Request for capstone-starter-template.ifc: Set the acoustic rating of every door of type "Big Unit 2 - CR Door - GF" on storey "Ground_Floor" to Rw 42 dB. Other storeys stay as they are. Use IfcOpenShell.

First a look at what the model holds.

```python
import ifcopenshell
import ifcopenshell.util.element

model = ifcopenshell.open("capstone-starter-template.ifc")
print(model.schema)
storey = next(s for s in model.by_type("IfcBuildingStorey") if s.Name == "Ground_Floor")
doors = [e for e in ifcopenshell.util.element.get_decomposition(storey) if e.is_a("IfcDoor")]
seen = {}
for e in doors:
    element_type = ifcopenshell.util.element.get_type(e)
    key = (element_type.Name if element_type != e and element_type else None, ifcopenshell.util.element.get_pset(e, "Pset_DoorCommon", "AcousticRating"))
    seen[key] = seen.get(key, 0) + 1
for (name, value), count in sorted(seen.items(), key=str):
    print(count, "x", name, "|", value)
```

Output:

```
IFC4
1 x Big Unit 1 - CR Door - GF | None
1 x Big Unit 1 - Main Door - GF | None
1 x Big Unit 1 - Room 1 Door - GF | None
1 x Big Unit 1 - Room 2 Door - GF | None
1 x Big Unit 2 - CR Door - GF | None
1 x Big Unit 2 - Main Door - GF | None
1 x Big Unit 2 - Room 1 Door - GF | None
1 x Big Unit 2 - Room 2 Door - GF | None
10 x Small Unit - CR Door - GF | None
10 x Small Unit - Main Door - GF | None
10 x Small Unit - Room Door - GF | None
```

```python
import ifcopenshell
import ifcopenshell.api.pset
import ifcopenshell.util.element

model = ifcopenshell.open("capstone-starter-template.ifc")

storey = next(s for s in model.by_type("IfcBuildingStorey") if s.Name == "Ground_Floor")
doors = [e for e in ifcopenshell.util.element.get_decomposition(storey) if e.is_a("IfcDoor")]

count = 0
for e in doors:
    element_type = ifcopenshell.util.element.get_type(e)
    if element_type in (None, e) or element_type.Name != "Big Unit 2 - CR Door - GF":
        continue
    # add_pset returns the element's existing set when there is one.
    pset = ifcopenshell.api.pset.add_pset(model, product=e, name="Pset_DoorCommon")
    ifcopenshell.api.pset.edit_pset(model, pset=pset, properties={"AcousticRating": "Rw 42 dB"})
    count += 1

print(count, "doors updated")

model.write("capstone-starter-template_edited.ifc")
```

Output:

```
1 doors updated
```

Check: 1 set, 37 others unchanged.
